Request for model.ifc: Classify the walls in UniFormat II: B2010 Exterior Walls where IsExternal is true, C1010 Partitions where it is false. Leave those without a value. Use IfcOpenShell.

First a look at what the model holds.

```python
import ifcopenshell
import ifcopenshell.util.element

model = ifcopenshell.open("model.ifc")
print(model.schema)
print("classifications:", [c.Name for c in model.by_type("IfcClassification")])
values = [ifcopenshell.util.element.get_pset(e, "Pset_WallCommon", "IsExternal") for e in model.by_type("IfcWall")]
for value in (True, False, None):
    print("IsExternal", value, values.count(value))
```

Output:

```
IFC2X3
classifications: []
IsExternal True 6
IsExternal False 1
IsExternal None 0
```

```python
import ifcopenshell
import ifcopenshell.api.classification
import ifcopenshell.util.element

model = ifcopenshell.open("model.ifc")

# IFC2X3 requires Source and Edition and has no link from the project to the system.
system = model.create_entity("IfcClassification", Source="ASTM", Edition="E1557", Name="UniFormat II")

walls = model.by_type("IfcWall")
external = {e: ifcopenshell.util.element.get_pset(e, "Pset_WallCommon", "IsExternal") for e in walls}
for flag, code, name in ((True, "B2010", "Exterior Walls"), (False, "C1010", "Partitions")):
    products = [e for e in walls if external[e] is flag]
    ifcopenshell.api.classification.add_reference(
        model, products=products, classification=system, identification=code, name=name
    )
    print(code, len(products))

model.write("model_rev.ifc")
```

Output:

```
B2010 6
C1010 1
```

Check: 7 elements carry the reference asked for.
